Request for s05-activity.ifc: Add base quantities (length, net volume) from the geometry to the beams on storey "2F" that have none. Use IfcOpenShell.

First a look at what the model holds.

```python
import ifcopenshell
import ifcopenshell.util.element
import ifcopenshell.util.unit

model = ifcopenshell.open("s05-activity.ifc")
print(model.schema)
for unit_type in ("LENGTHUNIT", "AREAUNIT", "VOLUMEUNIT"):
    print(unit_type, ifcopenshell.util.unit.calculate_unit_scale(model, unit_type))
storey = next(s for s in model.by_type("IfcBuildingStorey") if s.Name == "2F")
beams = [e for e in ifcopenshell.util.element.get_decomposition(storey) if e.is_a("IfcBeam")]
for e in sorted(beams, key=lambda e: e.id()):
    print(e.id(), e.is_a(), e.Name, list(ifcopenshell.util.element.get_psets(e, qtos_only=True)), sep=" | ")
```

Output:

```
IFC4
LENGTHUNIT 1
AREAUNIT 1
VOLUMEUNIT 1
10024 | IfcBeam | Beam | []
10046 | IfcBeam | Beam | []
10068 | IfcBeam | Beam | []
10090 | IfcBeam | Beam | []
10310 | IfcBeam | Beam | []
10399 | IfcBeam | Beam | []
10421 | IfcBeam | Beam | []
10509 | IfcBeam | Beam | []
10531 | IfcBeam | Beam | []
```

```python
import ifcopenshell
import ifcopenshell.api.pset
import ifcopenshell.geom
import ifcopenshell.util.element
import ifcopenshell.util.shape
import ifcopenshell.util.unit

model = ifcopenshell.open("s05-activity.ifc")
unit_scale = ifcopenshell.util.unit.calculate_unit_scale(model)
volume_scale = ifcopenshell.util.unit.calculate_unit_scale(model, "VOLUMEUNIT")
settings = ifcopenshell.geom.settings()

storey = next(s for s in model.by_type("IfcBuildingStorey") if s.Name == "2F")
beams = [e for e in ifcopenshell.util.element.get_decomposition(storey) if e.is_a("IfcBeam")]

for e in sorted(beams, key=lambda e: e.id()):
    if ifcopenshell.util.element.get_psets(e, qtos_only=True, should_inherit=False):
        continue
    # Geometry comes back in metres, in the element's own axes.
    shape = ifcopenshell.geom.create_shape(settings, e)
    values = {
        "Length": ifcopenshell.util.shape.get_max_xyz(shape.geometry) / unit_scale,
        "NetVolume": ifcopenshell.util.shape.get_volume(shape.geometry) / volume_scale,
    }
    qto = ifcopenshell.api.pset.add_qto(model, product=e, name="Qto_BeamBaseQuantities")
    ifcopenshell.api.pset.edit_qto(model, qto=qto, properties=values)
    print(e.id(), {k: round(v, 3) for k, v in values.items()})

model.write("s05-activity_rev.ifc")
```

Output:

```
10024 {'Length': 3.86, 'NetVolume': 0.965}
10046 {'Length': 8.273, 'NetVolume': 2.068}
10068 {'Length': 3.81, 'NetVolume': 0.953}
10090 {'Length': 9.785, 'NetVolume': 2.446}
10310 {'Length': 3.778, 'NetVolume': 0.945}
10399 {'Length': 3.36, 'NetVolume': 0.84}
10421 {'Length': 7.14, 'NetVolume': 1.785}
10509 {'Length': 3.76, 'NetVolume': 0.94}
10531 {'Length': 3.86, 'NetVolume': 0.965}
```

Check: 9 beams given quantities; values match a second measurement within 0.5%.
